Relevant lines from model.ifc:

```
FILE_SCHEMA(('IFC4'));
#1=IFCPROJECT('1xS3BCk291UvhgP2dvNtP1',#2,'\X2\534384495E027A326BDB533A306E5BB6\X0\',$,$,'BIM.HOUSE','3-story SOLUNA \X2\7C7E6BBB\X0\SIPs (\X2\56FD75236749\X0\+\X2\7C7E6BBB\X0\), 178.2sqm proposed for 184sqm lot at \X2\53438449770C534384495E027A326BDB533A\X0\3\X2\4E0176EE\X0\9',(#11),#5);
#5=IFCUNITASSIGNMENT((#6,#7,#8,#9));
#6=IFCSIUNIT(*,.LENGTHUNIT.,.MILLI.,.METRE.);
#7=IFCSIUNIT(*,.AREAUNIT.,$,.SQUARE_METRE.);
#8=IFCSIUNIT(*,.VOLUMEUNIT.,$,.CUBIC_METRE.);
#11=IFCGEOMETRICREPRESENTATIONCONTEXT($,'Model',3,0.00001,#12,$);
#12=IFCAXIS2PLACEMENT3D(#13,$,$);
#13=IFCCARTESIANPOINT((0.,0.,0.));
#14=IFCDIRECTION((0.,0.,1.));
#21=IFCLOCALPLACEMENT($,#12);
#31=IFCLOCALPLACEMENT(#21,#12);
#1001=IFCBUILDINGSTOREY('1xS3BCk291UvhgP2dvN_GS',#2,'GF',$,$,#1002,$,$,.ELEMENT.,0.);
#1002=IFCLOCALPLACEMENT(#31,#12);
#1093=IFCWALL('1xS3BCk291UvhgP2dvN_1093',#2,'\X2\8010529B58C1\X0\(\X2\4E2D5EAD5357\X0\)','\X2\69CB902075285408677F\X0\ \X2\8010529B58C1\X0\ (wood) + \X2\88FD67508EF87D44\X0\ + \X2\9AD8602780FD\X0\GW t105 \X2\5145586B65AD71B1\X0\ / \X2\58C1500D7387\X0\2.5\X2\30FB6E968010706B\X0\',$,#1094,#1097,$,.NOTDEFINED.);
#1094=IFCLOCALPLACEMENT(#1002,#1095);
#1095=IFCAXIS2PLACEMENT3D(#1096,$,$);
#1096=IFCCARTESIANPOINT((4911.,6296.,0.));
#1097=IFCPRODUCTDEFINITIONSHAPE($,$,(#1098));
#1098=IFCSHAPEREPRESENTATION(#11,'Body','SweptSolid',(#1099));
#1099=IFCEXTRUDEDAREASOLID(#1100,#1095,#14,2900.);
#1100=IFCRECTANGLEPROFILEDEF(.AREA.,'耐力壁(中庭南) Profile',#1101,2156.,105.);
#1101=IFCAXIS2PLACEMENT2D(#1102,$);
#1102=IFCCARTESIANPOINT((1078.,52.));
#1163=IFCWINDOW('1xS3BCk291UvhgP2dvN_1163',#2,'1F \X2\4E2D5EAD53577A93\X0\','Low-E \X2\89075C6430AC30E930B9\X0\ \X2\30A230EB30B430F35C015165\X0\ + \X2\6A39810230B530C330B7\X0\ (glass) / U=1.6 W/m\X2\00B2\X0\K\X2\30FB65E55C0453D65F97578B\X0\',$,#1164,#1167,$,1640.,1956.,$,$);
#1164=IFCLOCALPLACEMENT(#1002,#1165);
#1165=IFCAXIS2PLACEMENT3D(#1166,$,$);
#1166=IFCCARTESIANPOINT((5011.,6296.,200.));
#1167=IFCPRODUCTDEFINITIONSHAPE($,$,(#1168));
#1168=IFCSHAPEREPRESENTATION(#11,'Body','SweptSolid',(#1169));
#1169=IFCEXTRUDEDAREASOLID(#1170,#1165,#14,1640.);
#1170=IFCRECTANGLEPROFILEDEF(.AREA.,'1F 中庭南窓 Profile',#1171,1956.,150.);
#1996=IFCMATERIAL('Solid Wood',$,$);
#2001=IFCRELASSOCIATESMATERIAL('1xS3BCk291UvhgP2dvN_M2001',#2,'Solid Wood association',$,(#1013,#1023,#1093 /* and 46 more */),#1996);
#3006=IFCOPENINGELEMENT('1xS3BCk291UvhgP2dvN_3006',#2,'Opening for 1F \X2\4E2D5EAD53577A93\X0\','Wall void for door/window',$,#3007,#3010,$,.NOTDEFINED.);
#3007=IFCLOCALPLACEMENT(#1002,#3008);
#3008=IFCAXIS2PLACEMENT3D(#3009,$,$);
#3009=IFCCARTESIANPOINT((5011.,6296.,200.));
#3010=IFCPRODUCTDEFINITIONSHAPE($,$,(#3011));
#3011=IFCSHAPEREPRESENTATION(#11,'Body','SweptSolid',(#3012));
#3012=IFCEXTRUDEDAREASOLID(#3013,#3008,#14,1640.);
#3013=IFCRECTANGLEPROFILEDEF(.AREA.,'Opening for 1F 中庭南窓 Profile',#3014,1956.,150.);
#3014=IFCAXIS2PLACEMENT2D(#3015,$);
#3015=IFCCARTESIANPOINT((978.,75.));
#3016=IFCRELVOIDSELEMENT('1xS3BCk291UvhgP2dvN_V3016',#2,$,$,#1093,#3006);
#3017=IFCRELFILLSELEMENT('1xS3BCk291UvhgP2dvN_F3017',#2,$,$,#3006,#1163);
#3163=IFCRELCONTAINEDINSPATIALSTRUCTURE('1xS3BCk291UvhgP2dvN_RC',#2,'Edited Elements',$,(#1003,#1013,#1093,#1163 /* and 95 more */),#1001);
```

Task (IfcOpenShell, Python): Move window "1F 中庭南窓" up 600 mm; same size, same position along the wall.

```python
import numpy as np
import ifcopenshell
import ifcopenshell.api.geometry
import ifcopenshell.util.placement
import ifcopenshell.util.unit

model = ifcopenshell.open("model.ifc")
unit_scale = ifcopenshell.util.unit.calculate_unit_scale(model)

window = model.by_guid("1xS3BCk291UvhgP2dvN_1163")
opening = window.FillsVoids[0].RelatingOpeningElement
dz = 0.6 / unit_scale

shift = np.array([0.0, 0.0, dz])
# The window is not placed relative to its opening, so move both.
for product in (opening, window):
    matrix = ifcopenshell.util.placement.get_local_placement(product.ObjectPlacement)
    matrix[:3, 3] += shift
    ifcopenshell.api.geometry.edit_object_placement(model, product=product, matrix=matrix, is_si=False)

print(f"moved by {dz * unit_scale:+.3f} m")

model.write("model-out.ifc")
```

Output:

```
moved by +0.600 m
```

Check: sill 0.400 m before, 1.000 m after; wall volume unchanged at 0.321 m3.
